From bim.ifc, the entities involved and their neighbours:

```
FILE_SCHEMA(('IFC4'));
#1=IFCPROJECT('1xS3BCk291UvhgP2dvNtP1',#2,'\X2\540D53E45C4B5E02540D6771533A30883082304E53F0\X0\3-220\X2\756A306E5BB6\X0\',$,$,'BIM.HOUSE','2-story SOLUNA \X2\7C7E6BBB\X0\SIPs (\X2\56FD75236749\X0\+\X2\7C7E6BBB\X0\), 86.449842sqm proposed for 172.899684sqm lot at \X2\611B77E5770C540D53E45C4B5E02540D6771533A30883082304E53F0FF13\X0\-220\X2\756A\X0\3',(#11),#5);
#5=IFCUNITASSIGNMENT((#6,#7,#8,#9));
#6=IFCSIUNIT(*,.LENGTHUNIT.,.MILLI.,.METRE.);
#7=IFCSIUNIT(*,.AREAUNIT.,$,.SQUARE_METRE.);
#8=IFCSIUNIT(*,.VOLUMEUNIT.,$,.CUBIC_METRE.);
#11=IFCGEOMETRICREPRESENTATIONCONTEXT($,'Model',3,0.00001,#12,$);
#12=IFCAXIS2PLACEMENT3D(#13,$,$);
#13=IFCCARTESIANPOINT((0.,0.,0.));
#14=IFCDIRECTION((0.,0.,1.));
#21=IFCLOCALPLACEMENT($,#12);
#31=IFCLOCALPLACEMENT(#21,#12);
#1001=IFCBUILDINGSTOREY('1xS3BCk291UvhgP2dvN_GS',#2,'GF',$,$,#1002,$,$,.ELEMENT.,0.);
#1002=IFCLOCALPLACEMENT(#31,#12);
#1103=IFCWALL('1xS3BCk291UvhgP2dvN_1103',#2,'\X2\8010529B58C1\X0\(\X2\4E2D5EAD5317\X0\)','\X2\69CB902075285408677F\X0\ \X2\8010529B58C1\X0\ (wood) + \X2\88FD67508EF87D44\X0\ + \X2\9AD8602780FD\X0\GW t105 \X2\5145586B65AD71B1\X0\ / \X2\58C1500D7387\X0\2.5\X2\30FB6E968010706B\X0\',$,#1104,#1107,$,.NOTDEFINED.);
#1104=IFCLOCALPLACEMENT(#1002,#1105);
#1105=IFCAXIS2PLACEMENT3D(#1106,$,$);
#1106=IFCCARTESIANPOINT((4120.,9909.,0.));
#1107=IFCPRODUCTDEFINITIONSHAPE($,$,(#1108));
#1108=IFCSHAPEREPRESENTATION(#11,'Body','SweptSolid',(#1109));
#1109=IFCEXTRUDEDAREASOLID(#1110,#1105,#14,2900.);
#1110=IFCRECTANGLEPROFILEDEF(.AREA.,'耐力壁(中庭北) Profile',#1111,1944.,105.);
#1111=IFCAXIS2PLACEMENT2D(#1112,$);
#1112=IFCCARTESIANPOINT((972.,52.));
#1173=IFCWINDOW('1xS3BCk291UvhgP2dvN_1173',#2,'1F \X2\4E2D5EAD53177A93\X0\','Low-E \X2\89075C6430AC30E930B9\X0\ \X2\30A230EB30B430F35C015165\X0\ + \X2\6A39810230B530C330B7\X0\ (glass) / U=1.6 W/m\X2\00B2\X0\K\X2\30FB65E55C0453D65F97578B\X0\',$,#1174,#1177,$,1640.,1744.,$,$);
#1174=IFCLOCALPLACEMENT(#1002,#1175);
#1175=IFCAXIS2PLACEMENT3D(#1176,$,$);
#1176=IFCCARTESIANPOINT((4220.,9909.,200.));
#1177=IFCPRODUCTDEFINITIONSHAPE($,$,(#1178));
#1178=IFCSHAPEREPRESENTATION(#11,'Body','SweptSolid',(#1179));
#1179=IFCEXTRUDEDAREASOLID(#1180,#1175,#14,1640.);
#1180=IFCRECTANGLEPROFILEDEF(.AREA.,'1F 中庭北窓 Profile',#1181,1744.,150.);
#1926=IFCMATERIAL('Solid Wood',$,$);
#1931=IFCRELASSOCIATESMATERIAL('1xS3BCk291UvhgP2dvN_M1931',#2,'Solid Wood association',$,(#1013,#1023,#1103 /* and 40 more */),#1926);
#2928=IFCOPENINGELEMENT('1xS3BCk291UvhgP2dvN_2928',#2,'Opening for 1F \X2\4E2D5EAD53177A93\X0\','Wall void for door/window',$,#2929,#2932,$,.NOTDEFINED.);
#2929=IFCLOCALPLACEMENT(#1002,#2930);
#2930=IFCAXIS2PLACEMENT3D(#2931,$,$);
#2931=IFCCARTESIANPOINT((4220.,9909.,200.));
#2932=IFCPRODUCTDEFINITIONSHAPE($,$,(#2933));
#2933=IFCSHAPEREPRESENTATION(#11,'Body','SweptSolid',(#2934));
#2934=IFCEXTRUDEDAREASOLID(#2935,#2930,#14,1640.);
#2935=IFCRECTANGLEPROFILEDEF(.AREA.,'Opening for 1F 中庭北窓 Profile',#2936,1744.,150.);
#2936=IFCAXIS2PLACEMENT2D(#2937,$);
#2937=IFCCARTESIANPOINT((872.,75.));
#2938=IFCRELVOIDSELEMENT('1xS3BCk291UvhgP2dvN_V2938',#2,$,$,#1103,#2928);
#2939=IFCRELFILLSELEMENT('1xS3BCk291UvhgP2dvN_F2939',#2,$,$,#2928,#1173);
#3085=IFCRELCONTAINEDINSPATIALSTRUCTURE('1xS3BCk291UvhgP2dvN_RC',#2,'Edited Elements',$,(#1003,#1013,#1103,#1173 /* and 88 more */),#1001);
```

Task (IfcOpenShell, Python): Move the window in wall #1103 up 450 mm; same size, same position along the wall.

```python
import numpy as np
import ifcopenshell
import ifcopenshell.api.geometry
import ifcopenshell.util.placement
import ifcopenshell.util.unit

model = ifcopenshell.open("bim.ifc")
unit_scale = ifcopenshell.util.unit.calculate_unit_scale(model)

window = model.by_guid("1xS3BCk291UvhgP2dvN_1173")
opening = window.FillsVoids[0].RelatingOpeningElement
dz = 450.0

shift = np.array([0.0, 0.0, dz])
# The window is not placed relative to its opening, so move both.
for product in (opening, window):
    matrix = ifcopenshell.util.placement.get_local_placement(product.ObjectPlacement)
    matrix[:3, 3] += shift
    ifcopenshell.api.geometry.edit_object_placement(model, product=product, matrix=matrix, is_si=False)

print(f"moved by {dz * unit_scale:+.3f} m")

model.write("bim-out.ifc")
```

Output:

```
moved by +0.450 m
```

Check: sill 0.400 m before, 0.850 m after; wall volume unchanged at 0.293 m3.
